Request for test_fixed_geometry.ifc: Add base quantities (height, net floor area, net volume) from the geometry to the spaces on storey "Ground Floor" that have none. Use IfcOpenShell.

First a look at what the model holds.

```python
import ifcopenshell
import ifcopenshell.util.element
import ifcopenshell.util.unit

model = ifcopenshell.open("test_fixed_geometry.ifc")
print(model.schema)
for unit_type in ("LENGTHUNIT", "AREAUNIT", "VOLUMEUNIT"):
    print(unit_type, ifcopenshell.util.unit.calculate_unit_scale(model, unit_type))
storey = next(s for s in model.by_type("IfcBuildingStorey") if s.Name == "Ground Floor")
spaces = [e for e in ifcopenshell.util.element.get_decomposition(storey) if e.is_a("IfcSpace")]
for e in sorted(spaces, key=lambda e: e.id()):
    print(e.id(), e.is_a(), e.Name, list(ifcopenshell.util.element.get_psets(e, qtos_only=True)), sep=" | ")
```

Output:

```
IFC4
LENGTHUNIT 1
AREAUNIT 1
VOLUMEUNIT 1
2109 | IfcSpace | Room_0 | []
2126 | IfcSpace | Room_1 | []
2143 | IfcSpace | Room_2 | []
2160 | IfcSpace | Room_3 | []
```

```python
import ifcopenshell
import ifcopenshell.api.pset
import ifcopenshell.geom
import ifcopenshell.util.element
import ifcopenshell.util.shape
import ifcopenshell.util.unit

model = ifcopenshell.open("test_fixed_geometry.ifc")
unit_scale = ifcopenshell.util.unit.calculate_unit_scale(model)
area_scale = ifcopenshell.util.unit.calculate_unit_scale(model, "AREAUNIT")
volume_scale = ifcopenshell.util.unit.calculate_unit_scale(model, "VOLUMEUNIT")
settings = ifcopenshell.geom.settings()

storey = next(s for s in model.by_type("IfcBuildingStorey") if s.Name == "Ground Floor")
spaces = [e for e in ifcopenshell.util.element.get_decomposition(storey) if e.is_a("IfcSpace")]

for e in sorted(spaces, key=lambda e: e.id()):
    if ifcopenshell.util.element.get_psets(e, qtos_only=True, should_inherit=False):
        continue
    # Geometry comes back in metres, in the element's own axes.
    shape = ifcopenshell.geom.create_shape(settings, e)
    values = {
        "Height": ifcopenshell.util.shape.get_z(shape.geometry) / unit_scale,
        "NetFloorArea": ifcopenshell.util.shape.get_footprint_area(shape.geometry) / area_scale,
        "NetVolume": ifcopenshell.util.shape.get_volume(shape.geometry) / volume_scale,
    }
    qto = ifcopenshell.api.pset.add_qto(model, product=e, name="Qto_SpaceBaseQuantities")
    ifcopenshell.api.pset.edit_qto(model, qto=qto, properties=values)
    print(e.id(), {k: round(v, 3) for k, v in values.items()})

model.write("test_fixed_geometry_v2.ifc")
```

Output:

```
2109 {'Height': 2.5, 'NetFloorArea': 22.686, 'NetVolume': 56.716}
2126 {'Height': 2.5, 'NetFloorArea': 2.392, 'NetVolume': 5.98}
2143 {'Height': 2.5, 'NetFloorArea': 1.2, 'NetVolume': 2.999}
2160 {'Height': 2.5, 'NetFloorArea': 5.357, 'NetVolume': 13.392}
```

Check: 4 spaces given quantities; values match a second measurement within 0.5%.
